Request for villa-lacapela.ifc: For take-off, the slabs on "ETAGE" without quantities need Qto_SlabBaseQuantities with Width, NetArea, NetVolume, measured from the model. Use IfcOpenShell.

First a look at what the model holds.

```python
import ifcopenshell
import ifcopenshell.util.element
import ifcopenshell.util.unit

model = ifcopenshell.open("villa-lacapela.ifc")
print(model.schema)
for unit_type in ("LENGTHUNIT", "AREAUNIT", "VOLUMEUNIT"):
    print(unit_type, ifcopenshell.util.unit.calculate_unit_scale(model, unit_type))
storey = next(s for s in model.by_type("IfcBuildingStorey") if s.Name == "ETAGE")
slabs = [e for e in ifcopenshell.util.element.get_decomposition(storey) if e.is_a("IfcSlab")]
for e in sorted(slabs, key=lambda e: e.id()):
    print(e.id(), e.is_a(), e.Name, list(ifcopenshell.util.element.get_psets(e, qtos_only=True)), sep=" | ")
```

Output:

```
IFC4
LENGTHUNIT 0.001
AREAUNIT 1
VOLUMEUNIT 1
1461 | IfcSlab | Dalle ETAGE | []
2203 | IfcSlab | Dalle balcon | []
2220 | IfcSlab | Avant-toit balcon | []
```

```python
import ifcopenshell
import ifcopenshell.api.pset
import ifcopenshell.geom
import ifcopenshell.util.element
import ifcopenshell.util.shape
import ifcopenshell.util.unit

model = ifcopenshell.open("villa-lacapela.ifc")
unit_scale = ifcopenshell.util.unit.calculate_unit_scale(model)
area_scale = ifcopenshell.util.unit.calculate_unit_scale(model, "AREAUNIT")
volume_scale = ifcopenshell.util.unit.calculate_unit_scale(model, "VOLUMEUNIT")
settings = ifcopenshell.geom.settings()

storey = next(s for s in model.by_type("IfcBuildingStorey") if s.Name == "ETAGE")
slabs = [e for e in ifcopenshell.util.element.get_decomposition(storey) if e.is_a("IfcSlab")]

for e in sorted(slabs, key=lambda e: e.id()):
    if ifcopenshell.util.element.get_psets(e, qtos_only=True, should_inherit=False):
        continue
    # Geometry comes back in metres, in the element's own axes.
    shape = ifcopenshell.geom.create_shape(settings, e)
    values = {
        "Width": ifcopenshell.util.shape.get_z(shape.geometry) / unit_scale,
        "NetArea": ifcopenshell.util.shape.get_footprint_area(shape.geometry) / area_scale,
        "NetVolume": ifcopenshell.util.shape.get_volume(shape.geometry) / volume_scale,
    }
    qto = ifcopenshell.api.pset.add_qto(model, product=e, name="Qto_SlabBaseQuantities")
    ifcopenshell.api.pset.edit_qto(model, qto=qto, properties=values)
    print(e.id(), {k: round(v, 3) for k, v in values.items()})

model.write("villa-lacapela_v2.ifc")
```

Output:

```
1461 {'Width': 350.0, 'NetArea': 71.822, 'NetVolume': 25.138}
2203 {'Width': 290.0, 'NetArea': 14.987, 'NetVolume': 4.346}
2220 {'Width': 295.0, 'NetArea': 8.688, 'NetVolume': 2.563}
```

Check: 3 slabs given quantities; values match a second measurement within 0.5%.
